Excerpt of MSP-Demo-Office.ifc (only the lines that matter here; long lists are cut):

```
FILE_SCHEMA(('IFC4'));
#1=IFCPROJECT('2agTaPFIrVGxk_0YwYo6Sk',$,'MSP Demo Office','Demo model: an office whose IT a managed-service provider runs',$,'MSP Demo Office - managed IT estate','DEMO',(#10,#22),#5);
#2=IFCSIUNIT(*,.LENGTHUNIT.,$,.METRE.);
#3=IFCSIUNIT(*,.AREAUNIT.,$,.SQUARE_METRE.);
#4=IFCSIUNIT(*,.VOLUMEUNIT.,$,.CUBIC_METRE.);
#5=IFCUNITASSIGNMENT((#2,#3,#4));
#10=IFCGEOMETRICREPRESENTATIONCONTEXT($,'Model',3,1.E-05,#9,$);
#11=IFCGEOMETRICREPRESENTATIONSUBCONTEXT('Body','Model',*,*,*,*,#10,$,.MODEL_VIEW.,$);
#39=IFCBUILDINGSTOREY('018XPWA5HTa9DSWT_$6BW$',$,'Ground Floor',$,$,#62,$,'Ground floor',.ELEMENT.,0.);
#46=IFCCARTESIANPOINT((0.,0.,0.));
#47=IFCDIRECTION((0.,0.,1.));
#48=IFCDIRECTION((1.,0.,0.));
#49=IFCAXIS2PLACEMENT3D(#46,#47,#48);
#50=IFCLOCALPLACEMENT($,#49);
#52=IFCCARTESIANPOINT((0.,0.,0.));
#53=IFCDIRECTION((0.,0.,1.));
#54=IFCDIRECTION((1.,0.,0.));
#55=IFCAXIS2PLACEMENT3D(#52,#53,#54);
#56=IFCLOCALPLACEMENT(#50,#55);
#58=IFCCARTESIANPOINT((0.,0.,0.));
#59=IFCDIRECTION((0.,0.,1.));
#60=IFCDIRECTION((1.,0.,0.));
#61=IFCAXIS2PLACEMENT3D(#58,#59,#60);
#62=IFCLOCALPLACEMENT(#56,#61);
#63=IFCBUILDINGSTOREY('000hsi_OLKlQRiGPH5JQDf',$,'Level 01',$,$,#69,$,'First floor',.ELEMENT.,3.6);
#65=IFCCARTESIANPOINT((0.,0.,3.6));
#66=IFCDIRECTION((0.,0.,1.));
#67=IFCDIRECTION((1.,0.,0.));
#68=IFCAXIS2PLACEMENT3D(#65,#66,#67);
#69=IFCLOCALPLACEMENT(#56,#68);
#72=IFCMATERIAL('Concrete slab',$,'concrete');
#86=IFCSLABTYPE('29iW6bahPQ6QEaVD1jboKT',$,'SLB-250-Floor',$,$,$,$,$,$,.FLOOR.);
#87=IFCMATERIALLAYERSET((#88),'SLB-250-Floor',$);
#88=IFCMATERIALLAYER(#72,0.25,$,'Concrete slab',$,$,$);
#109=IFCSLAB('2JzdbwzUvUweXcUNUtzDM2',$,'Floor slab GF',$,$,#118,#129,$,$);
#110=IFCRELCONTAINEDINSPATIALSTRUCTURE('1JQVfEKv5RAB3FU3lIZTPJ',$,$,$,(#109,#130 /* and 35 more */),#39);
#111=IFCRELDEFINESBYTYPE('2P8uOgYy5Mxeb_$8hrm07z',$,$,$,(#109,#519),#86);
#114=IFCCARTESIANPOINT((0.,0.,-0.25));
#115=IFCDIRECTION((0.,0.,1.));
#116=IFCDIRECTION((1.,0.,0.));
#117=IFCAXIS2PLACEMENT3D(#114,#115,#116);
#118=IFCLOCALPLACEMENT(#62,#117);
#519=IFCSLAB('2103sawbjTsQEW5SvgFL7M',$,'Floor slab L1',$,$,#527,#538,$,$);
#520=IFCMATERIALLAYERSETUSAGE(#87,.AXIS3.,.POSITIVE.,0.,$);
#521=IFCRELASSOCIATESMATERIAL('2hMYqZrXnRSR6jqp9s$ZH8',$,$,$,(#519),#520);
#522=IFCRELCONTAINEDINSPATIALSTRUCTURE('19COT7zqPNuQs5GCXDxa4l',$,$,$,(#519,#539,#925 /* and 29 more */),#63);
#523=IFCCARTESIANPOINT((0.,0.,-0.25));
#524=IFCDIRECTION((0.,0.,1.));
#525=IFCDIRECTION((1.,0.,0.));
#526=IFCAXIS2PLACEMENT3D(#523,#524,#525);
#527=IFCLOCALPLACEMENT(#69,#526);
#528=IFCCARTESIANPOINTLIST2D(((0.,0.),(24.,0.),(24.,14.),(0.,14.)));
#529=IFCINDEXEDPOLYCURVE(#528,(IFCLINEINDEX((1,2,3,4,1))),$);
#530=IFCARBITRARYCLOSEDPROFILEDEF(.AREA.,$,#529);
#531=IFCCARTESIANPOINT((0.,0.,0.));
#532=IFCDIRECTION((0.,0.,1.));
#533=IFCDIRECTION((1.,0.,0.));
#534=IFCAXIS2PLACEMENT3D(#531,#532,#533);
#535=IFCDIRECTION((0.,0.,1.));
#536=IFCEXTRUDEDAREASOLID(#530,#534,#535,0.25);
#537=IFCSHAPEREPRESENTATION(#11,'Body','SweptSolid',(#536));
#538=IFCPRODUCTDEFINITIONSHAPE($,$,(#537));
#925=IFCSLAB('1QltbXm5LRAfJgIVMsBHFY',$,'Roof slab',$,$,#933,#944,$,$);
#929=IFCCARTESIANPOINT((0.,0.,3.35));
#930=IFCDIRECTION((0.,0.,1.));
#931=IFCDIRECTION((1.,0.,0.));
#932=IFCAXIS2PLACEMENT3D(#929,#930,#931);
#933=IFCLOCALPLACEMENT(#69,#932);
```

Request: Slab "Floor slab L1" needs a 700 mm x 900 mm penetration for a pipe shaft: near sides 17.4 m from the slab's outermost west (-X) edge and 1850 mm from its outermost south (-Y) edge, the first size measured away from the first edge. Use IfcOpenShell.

```python
import numpy as np
import ifcopenshell
import ifcopenshell.api.feature
import ifcopenshell.api.geometry
import ifcopenshell.api.root
import ifcopenshell.geom
import ifcopenshell.util.placement
import ifcopenshell.util.representation
import ifcopenshell.util.shape
import ifcopenshell.util.unit

model = ifcopenshell.open("MSP-Demo-Office.ifc")
unit_scale = ifcopenshell.util.unit.calculate_unit_scale(model)
settings = ifcopenshell.geom.settings()


def volume(element):
    """Net volume in cubic metres, openings subtracted."""
    shape = ifcopenshell.geom.create_shape(settings, element)
    return ifcopenshell.util.shape.get_volume(shape.geometry)


slab = model.by_guid("2103sawbjTsQEW5SvgFL7M")
before = volume(slab)

# Extent in the slab's own axes, in metres. The edges named are its -X and -Y sides.
slab_shape = ifcopenshell.geom.create_shape(settings, slab)
vertices = ifcopenshell.util.shape.get_vertices(slab_shape.geometry)
x_min, y_min, bottom = vertices.min(axis=0)
top = vertices[:, 2].max()

opening = ifcopenshell.api.root.create_entity(model, ifc_class="IfcOpeningElement", name="Pipe shaft opening", predefined_type="OPENING")
context = ifcopenshell.util.representation.get_context(model, "Model", "Body", "MODEL_VIEW")
width, depth = 0.7, 0.9
outline = [(0.0, 0.0), (width, 0.0), (width, depth), (0.0, depth), (0.0, 0.0)]
# Overshoot both faces by 50 mm so the cut is clean.
shape = ifcopenshell.api.geometry.add_slab_representation(
    model, context=context, depth=top - bottom + 0.1, polyline=outline
)
ifcopenshell.api.geometry.assign_representation(model, product=opening, representation=shape)

matrix = ifcopenshell.util.placement.get_local_placement(slab.ObjectPlacement)
matrix[:, 3] = matrix @ np.append(np.array([x_min + 17.4, y_min + 1.85, bottom - 0.05]) / unit_scale, 1.0)
ifcopenshell.api.geometry.edit_object_placement(model, product=opening, matrix=matrix, is_si=False)
ifcopenshell.api.feature.add_feature(model, feature=opening, element=slab)

after = volume(slab)

print(f"slab volume {before:.3f} -> {after:.3f} m3")

model.write("MSP-Demo-Office_edited.ifc")
```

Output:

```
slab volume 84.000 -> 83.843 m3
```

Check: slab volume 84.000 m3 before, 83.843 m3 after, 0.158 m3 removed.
